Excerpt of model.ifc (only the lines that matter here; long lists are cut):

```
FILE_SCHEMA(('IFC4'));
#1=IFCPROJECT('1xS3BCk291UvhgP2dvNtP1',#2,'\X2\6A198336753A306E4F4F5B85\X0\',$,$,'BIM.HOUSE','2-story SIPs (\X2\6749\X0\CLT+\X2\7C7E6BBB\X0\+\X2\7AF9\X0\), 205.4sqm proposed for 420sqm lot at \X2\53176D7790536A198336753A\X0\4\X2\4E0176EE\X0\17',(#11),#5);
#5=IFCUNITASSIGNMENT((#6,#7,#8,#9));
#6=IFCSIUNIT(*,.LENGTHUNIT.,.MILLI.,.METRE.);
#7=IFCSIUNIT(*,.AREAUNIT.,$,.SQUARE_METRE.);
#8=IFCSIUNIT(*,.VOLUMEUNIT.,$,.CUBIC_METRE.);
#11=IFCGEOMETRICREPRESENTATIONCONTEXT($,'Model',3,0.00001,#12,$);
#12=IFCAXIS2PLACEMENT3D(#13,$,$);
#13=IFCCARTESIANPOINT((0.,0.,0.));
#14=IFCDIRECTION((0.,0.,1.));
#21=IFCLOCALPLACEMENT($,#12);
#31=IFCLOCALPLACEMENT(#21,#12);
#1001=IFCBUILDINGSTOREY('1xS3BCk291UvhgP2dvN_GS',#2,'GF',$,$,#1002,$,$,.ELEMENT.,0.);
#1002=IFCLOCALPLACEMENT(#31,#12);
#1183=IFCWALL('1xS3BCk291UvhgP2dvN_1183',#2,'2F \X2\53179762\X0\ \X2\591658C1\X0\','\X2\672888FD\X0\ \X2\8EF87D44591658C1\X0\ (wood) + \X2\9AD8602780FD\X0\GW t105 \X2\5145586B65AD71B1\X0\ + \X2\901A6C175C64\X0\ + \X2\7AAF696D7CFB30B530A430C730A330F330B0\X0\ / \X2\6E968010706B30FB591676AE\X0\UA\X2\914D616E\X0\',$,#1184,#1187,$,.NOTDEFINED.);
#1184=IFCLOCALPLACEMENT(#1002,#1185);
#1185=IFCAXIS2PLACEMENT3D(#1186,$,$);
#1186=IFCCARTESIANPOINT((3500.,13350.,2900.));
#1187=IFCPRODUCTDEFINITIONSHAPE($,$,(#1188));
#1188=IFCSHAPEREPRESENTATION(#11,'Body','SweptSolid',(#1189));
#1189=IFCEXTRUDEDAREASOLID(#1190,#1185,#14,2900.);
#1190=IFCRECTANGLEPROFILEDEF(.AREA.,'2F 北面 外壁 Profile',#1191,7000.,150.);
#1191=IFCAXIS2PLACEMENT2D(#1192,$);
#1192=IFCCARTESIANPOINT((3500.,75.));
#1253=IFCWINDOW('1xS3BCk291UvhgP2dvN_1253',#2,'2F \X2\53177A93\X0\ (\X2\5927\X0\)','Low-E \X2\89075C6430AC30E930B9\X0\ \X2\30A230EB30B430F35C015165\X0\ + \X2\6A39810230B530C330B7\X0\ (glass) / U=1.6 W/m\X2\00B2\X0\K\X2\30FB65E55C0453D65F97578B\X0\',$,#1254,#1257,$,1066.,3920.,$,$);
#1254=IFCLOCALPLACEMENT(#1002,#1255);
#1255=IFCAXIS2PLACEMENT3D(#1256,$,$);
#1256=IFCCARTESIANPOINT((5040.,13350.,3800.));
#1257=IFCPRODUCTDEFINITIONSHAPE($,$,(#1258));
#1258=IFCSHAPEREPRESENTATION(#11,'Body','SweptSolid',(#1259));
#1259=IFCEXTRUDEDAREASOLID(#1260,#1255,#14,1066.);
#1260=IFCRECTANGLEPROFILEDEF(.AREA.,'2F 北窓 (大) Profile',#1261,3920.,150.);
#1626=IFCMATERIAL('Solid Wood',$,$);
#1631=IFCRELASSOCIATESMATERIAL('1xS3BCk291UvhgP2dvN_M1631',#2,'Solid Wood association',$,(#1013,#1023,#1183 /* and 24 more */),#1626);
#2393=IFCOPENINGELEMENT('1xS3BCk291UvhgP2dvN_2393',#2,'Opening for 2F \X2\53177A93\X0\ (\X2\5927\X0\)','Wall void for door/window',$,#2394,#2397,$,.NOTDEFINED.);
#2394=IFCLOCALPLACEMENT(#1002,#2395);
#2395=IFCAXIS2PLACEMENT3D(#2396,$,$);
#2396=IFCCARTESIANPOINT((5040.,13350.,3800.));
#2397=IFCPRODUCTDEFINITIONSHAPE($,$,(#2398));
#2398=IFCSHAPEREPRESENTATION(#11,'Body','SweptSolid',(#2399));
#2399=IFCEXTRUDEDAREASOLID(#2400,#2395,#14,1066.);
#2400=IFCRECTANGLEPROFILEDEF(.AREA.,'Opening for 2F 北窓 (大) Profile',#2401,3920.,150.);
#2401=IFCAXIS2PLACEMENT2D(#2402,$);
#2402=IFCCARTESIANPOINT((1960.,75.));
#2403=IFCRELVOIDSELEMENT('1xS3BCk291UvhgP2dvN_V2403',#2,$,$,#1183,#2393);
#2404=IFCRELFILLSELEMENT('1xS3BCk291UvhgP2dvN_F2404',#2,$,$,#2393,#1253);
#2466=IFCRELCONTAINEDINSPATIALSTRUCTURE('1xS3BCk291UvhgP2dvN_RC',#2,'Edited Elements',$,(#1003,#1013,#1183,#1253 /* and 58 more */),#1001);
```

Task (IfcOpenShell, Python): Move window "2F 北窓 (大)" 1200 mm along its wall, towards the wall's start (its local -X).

```python
import ifcopenshell
import ifcopenshell.api.geometry
import ifcopenshell.util.placement
import ifcopenshell.util.unit

model = ifcopenshell.open("model.ifc")
unit_scale = ifcopenshell.util.unit.calculate_unit_scale(model)

window = model.by_guid("1xS3BCk291UvhgP2dvN_1253")
opening = window.FillsVoids[0].RelatingOpeningElement
wall = opening.VoidsElements[0].RelatingBuildingElement

wall_matrix = ifcopenshell.util.placement.get_local_placement(wall.ObjectPlacement)
shift = wall_matrix[:3, 0] * -1.2 / unit_scale
before = ifcopenshell.util.placement.get_local_placement(window.ObjectPlacement)[:3, 3].copy()

# The window is not placed relative to its opening, so move both.
for product in (opening, window):
    matrix = ifcopenshell.util.placement.get_local_placement(product.ObjectPlacement)
    matrix[:3, 3] += shift
    ifcopenshell.api.geometry.edit_object_placement(model, product=product, matrix=matrix, is_si=False)

after = ifcopenshell.util.placement.get_local_placement(window.ObjectPlacement)[:3, 3]
print("window moved by", (after - before).round(3) + 0.0)

model.write("model_rev.ifc")
```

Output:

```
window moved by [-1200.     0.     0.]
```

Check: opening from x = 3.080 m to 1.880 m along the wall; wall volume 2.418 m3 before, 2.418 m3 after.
